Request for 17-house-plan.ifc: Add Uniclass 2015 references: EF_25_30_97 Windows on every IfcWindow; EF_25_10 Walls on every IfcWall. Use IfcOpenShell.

First a look at what the model holds.

```python
import ifcopenshell

model = ifcopenshell.open("17-house-plan.ifc")
print(model.schema)
print("classifications:", [c.Name for c in model.by_type("IfcClassification")])
for ifc_class in ("IfcDoor", "IfcRoof", "IfcStair", "IfcWall", "IfcWindow"):
    print(ifc_class, len(model.by_type(ifc_class)))
```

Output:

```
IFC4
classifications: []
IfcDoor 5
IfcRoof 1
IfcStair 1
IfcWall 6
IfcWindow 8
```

```python
import ifcopenshell
import ifcopenshell.api.classification

model = ifcopenshell.open("17-house-plan.ifc")

system = ifcopenshell.api.classification.add_classification(model, classification="Uniclass 2015")

codes = {
    "IfcWindow": ("EF_25_30_97", "Windows"),
    "IfcWall": ("EF_25_10", "Walls"),
}
for ifc_class, (code, name) in codes.items():
    products = model.by_type(ifc_class)
    ifcopenshell.api.classification.add_reference(
        model, products=products, classification=system, identification=code, name=name
    )
    print(code, len(products))

model.write("17-house-plan_rev.ifc")
```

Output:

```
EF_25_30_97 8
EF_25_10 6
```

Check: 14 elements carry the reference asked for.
